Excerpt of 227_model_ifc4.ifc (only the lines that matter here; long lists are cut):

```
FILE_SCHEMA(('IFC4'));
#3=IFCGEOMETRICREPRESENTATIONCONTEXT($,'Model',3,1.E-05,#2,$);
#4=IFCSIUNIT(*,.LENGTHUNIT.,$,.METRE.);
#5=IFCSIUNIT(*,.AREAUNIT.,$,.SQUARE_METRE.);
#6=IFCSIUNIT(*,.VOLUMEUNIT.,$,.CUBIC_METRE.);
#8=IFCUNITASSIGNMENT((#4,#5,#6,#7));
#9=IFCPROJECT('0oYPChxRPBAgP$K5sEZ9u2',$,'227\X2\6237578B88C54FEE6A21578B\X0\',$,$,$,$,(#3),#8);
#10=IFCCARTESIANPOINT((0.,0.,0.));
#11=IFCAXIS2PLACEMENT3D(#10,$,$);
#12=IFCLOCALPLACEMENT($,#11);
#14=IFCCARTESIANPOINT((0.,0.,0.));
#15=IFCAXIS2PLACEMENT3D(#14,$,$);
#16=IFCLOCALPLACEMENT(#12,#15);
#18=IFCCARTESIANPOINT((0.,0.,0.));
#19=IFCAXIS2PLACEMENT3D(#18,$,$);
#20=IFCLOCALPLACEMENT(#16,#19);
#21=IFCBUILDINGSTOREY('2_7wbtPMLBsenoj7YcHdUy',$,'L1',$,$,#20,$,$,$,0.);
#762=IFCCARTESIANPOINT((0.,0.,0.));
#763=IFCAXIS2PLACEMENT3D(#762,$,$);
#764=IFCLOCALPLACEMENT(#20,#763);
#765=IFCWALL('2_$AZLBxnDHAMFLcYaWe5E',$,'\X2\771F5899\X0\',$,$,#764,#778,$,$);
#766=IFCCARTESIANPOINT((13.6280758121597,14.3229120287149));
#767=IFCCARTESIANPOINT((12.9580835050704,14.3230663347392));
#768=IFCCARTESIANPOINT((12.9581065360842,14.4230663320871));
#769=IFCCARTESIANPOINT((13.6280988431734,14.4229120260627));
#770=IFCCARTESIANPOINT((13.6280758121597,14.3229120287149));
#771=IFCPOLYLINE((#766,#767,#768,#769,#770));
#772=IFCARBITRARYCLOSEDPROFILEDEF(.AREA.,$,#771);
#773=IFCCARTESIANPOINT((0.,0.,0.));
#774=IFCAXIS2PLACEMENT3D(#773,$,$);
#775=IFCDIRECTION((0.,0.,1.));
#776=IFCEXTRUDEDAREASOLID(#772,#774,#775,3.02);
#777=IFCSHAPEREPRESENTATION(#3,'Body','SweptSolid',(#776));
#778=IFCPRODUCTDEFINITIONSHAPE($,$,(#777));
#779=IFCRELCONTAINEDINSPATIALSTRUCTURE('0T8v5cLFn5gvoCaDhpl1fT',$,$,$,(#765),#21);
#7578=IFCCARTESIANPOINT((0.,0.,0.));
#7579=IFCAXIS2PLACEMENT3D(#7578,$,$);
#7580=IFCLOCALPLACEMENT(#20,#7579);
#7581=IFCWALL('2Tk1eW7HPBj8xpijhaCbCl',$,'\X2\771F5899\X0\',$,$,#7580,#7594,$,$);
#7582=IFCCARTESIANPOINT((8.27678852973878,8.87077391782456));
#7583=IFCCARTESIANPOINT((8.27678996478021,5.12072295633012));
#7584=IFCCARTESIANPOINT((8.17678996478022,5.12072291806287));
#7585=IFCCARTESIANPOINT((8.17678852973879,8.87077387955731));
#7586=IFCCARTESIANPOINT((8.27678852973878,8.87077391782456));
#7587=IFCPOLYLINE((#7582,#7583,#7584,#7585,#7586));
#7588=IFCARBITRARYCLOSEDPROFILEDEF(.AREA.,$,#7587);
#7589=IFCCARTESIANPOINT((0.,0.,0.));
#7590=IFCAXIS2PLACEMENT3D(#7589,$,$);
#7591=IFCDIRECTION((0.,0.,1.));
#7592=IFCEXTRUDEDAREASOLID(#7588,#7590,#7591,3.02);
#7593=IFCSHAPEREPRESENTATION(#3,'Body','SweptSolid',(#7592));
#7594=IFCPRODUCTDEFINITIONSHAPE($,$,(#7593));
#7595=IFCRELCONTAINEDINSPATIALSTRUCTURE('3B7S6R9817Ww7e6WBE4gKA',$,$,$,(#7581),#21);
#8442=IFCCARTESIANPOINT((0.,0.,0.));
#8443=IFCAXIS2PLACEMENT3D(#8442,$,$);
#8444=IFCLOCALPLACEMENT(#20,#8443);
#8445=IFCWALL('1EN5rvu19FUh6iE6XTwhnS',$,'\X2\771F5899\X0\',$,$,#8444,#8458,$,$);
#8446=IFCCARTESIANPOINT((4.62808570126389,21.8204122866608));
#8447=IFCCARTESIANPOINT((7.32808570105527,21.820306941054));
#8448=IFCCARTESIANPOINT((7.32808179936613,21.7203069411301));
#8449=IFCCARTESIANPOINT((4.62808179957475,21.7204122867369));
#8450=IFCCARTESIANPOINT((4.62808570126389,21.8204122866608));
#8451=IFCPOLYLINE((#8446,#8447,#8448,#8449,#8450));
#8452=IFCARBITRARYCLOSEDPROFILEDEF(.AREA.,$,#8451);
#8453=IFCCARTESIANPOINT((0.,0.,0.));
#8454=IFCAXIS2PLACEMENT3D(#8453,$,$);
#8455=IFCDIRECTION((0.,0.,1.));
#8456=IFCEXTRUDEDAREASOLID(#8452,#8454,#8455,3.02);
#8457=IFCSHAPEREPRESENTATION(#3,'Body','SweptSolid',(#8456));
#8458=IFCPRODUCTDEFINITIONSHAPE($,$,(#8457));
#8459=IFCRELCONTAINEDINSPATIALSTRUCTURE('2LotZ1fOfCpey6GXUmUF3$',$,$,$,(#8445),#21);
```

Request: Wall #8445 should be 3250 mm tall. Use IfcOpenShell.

```python
import ifcopenshell
import ifcopenshell.geom
import ifcopenshell.util.shape
import ifcopenshell.util.unit

model = ifcopenshell.open("227_model_ifc4.ifc")
unit_scale = ifcopenshell.util.unit.calculate_unit_scale(model)
settings = ifcopenshell.geom.settings()


def volume(element):
    """Net volume in cubic metres, openings subtracted."""
    shape = ifcopenshell.geom.create_shape(settings, element)
    return ifcopenshell.util.shape.get_volume(shape.geometry)


wall = model.by_id(8445)
before = volume(wall)

body = next(r for r in wall.Representation.Representations if r.RepresentationIdentifier == "Body")
solid = body.Items[0]
old_height = solid.Depth
solid.Depth = 3.25 / unit_scale
after = volume(wall)

print(f"height {old_height:g} -> {solid.Depth:g}, volume {before:.3f} -> {after:.3f} m3")

model.write("227_model_ifc4_updated.ifc")
```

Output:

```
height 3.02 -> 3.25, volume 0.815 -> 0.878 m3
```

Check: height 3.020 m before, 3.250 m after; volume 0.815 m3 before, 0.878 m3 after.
